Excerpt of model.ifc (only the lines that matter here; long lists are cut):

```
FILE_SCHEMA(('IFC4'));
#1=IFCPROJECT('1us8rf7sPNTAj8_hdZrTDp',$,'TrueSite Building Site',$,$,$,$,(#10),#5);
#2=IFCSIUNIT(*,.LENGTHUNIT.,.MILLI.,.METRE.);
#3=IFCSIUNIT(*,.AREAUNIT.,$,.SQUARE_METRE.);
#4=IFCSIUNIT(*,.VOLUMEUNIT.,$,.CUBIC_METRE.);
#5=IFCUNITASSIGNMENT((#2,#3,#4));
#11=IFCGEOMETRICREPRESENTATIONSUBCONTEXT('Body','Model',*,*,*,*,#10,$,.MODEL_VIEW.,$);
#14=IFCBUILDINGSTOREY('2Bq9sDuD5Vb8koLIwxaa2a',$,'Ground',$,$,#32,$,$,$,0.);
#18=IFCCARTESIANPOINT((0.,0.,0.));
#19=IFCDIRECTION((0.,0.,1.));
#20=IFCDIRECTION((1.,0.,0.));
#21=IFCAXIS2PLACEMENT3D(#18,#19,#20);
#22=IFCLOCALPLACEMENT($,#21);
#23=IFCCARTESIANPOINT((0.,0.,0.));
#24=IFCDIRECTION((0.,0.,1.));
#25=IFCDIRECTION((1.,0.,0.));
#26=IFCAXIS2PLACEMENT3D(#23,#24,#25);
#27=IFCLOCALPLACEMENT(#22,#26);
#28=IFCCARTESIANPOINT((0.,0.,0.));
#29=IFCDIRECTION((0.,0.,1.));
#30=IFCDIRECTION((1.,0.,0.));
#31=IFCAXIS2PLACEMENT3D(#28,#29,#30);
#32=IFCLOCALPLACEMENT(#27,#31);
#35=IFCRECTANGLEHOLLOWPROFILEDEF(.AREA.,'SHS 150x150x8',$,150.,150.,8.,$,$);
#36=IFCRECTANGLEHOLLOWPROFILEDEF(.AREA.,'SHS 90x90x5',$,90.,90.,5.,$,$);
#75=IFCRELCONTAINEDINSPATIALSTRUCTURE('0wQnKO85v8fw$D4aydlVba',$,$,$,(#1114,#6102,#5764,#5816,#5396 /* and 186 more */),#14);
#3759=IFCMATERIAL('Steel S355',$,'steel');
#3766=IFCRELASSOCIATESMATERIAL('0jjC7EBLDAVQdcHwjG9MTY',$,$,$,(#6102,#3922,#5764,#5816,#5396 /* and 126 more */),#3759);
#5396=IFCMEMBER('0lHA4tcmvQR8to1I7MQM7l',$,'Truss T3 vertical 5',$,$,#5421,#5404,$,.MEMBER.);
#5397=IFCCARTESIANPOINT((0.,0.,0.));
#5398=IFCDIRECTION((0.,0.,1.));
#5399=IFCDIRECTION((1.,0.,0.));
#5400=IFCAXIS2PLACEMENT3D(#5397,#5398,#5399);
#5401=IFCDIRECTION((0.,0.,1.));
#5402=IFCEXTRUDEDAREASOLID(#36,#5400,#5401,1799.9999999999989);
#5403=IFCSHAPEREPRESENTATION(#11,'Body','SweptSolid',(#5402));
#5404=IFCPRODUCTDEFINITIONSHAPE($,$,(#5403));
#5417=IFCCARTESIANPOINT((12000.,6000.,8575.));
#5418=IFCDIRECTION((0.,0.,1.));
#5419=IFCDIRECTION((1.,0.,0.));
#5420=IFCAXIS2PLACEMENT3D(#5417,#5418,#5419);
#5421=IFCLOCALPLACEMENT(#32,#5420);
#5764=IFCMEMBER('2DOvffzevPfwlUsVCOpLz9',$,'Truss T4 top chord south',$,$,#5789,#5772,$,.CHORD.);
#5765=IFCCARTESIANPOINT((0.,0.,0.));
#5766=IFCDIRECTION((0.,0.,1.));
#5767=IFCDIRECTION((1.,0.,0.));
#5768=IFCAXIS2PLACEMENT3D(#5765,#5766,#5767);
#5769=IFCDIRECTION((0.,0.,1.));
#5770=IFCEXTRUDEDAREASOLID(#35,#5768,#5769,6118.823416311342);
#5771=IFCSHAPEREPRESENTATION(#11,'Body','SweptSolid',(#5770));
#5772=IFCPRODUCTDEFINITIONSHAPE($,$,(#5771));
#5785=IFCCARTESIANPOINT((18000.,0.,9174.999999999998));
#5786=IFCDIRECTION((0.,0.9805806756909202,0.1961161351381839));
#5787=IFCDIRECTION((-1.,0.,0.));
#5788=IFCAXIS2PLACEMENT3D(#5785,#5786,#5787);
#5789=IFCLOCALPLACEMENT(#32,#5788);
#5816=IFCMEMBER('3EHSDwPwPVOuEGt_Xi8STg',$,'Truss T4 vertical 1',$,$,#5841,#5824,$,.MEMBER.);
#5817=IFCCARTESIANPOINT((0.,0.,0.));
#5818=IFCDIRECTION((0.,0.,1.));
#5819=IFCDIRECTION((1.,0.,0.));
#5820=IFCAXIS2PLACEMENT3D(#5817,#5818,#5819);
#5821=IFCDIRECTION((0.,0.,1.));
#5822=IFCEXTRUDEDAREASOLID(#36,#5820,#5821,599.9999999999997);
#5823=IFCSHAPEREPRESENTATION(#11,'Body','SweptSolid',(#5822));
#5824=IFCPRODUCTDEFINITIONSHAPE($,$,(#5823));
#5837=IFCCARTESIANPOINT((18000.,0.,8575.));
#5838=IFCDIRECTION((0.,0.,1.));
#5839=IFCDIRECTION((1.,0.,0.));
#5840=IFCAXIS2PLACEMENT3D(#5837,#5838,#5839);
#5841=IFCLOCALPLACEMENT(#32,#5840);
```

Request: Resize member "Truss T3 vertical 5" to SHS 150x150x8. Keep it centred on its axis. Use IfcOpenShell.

```python
import ifcopenshell
import ifcopenshell.util.element
import ifcopenshell.util.representation

model = ifcopenshell.open("model.ifc")

member = model.by_guid("0lHA4tcmvQR8to1I7MQM7l")
source = next(p for p in model.by_type("IfcRectangleHollowProfileDef") if p.ProfileName == "SHS 150x150x8")

body = ifcopenshell.util.representation.get_representation(member, "Model", "Body")
solid = body.Items[0]
old_profile = solid.SweptArea

# Copy the section's sizes but keep this member's own profile position.
profile = ifcopenshell.util.element.copy(model, source)
profile.Position = old_profile.Position
solid.SweptArea = profile
if not model.get_total_inverses(old_profile):
    ifcopenshell.util.element.remove_deep2(model, old_profile)

print(solid.SweptArea)

model.write("model-out.ifc")
```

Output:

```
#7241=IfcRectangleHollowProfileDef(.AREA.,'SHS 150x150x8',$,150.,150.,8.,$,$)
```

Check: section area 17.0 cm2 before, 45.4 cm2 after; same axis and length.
